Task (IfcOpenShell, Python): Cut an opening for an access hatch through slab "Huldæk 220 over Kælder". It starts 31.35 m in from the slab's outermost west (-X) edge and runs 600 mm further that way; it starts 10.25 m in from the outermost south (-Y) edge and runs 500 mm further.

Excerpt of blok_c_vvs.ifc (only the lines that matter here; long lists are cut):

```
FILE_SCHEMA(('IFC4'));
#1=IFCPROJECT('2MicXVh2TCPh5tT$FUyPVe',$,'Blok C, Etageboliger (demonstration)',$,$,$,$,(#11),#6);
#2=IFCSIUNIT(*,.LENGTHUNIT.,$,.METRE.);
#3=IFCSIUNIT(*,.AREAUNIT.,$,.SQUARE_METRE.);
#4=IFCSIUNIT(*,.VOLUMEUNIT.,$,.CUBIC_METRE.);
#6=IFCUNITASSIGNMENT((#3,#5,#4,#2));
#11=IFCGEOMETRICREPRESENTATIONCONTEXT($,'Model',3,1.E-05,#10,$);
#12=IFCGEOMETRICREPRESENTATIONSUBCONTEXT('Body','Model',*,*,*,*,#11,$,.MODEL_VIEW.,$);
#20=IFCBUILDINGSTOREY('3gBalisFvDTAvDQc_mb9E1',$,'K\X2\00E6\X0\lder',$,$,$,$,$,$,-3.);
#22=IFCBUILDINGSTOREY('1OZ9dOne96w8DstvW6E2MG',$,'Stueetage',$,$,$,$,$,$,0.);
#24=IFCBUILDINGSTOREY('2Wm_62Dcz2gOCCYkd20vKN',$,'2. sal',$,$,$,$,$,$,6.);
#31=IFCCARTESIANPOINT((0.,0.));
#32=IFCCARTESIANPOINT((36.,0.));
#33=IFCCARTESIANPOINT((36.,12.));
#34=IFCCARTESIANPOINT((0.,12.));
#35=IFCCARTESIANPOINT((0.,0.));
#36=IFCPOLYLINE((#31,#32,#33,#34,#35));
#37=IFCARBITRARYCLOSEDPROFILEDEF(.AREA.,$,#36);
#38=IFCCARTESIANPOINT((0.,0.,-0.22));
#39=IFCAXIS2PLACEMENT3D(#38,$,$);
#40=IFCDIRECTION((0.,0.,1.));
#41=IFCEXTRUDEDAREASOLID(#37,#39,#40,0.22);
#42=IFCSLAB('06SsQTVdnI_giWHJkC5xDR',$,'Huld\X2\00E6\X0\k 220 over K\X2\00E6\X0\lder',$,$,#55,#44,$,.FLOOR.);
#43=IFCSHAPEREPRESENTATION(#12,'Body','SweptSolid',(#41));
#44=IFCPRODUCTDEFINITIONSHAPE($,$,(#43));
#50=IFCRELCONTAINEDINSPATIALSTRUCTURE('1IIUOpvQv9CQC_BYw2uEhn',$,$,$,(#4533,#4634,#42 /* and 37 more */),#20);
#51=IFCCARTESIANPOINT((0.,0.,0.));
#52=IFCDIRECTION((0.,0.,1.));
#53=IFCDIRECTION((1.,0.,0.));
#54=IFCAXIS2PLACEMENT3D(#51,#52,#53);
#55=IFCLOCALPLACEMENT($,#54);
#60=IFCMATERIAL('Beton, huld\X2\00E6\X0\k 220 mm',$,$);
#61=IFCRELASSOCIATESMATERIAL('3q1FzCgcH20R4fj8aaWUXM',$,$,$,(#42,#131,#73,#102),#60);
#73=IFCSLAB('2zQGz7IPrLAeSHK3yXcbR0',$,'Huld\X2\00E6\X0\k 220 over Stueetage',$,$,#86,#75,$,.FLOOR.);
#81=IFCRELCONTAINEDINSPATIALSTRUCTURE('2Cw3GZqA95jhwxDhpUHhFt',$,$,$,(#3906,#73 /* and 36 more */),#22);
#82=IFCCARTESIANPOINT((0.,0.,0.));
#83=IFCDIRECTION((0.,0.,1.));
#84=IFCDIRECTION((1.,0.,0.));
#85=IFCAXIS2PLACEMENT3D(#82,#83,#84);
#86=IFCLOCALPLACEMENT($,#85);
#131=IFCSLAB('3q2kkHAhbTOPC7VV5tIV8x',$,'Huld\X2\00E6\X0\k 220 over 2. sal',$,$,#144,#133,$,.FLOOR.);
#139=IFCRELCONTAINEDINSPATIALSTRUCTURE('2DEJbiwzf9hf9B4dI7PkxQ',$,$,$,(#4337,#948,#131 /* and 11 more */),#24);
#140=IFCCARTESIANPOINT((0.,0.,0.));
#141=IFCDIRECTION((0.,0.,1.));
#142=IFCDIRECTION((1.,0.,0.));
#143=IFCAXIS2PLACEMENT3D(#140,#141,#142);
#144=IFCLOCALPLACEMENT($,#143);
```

```python
import numpy as np
import ifcopenshell
import ifcopenshell.api.feature
import ifcopenshell.api.geometry
import ifcopenshell.api.root
import ifcopenshell.geom
import ifcopenshell.util.placement
import ifcopenshell.util.representation
import ifcopenshell.util.shape
import ifcopenshell.util.unit

model = ifcopenshell.open("blok_c_vvs.ifc")
unit_scale = ifcopenshell.util.unit.calculate_unit_scale(model)
settings = ifcopenshell.geom.settings()


def volume(element):
    """Net volume in cubic metres, openings subtracted."""
    shape = ifcopenshell.geom.create_shape(settings, element)
    return ifcopenshell.util.shape.get_volume(shape.geometry)


slab = model.by_guid("06SsQTVdnI_giWHJkC5xDR")
before = volume(slab)

# Extent in the slab's own axes, in metres. The edges named are its -X and -Y sides.
slab_shape = ifcopenshell.geom.create_shape(settings, slab)
vertices = ifcopenshell.util.shape.get_vertices(slab_shape.geometry)
x_min, y_min, bottom = vertices.min(axis=0)
top = vertices[:, 2].max()

opening = ifcopenshell.api.root.create_entity(model, ifc_class="IfcOpeningElement", name="Access hatch opening", predefined_type="OPENING")
context = ifcopenshell.util.representation.get_context(model, "Model", "Body", "MODEL_VIEW")
width, depth = 0.6, 0.5
outline = [(0.0, 0.0), (width, 0.0), (width, depth), (0.0, depth), (0.0, 0.0)]
# Overshoot both faces by 50 mm so the cut is clean.
shape = ifcopenshell.api.geometry.add_slab_representation(
    model, context=context, depth=top - bottom + 0.1, polyline=outline
)
ifcopenshell.api.geometry.assign_representation(model, product=opening, representation=shape)

matrix = ifcopenshell.util.placement.get_local_placement(slab.ObjectPlacement)
matrix[:, 3] = matrix @ np.append(np.array([x_min + 31.35, y_min + 10.25, bottom - 0.05]) / unit_scale, 1.0)
ifcopenshell.api.geometry.edit_object_placement(model, product=opening, matrix=matrix, is_si=False)
ifcopenshell.api.feature.add_feature(model, feature=opening, element=slab)

after = volume(slab)

print(f"slab volume {before:.3f} -> {after:.3f} m3")

model.write("blok_c_vvs_v2.ifc")
```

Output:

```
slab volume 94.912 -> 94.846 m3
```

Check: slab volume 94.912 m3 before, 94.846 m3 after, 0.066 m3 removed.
